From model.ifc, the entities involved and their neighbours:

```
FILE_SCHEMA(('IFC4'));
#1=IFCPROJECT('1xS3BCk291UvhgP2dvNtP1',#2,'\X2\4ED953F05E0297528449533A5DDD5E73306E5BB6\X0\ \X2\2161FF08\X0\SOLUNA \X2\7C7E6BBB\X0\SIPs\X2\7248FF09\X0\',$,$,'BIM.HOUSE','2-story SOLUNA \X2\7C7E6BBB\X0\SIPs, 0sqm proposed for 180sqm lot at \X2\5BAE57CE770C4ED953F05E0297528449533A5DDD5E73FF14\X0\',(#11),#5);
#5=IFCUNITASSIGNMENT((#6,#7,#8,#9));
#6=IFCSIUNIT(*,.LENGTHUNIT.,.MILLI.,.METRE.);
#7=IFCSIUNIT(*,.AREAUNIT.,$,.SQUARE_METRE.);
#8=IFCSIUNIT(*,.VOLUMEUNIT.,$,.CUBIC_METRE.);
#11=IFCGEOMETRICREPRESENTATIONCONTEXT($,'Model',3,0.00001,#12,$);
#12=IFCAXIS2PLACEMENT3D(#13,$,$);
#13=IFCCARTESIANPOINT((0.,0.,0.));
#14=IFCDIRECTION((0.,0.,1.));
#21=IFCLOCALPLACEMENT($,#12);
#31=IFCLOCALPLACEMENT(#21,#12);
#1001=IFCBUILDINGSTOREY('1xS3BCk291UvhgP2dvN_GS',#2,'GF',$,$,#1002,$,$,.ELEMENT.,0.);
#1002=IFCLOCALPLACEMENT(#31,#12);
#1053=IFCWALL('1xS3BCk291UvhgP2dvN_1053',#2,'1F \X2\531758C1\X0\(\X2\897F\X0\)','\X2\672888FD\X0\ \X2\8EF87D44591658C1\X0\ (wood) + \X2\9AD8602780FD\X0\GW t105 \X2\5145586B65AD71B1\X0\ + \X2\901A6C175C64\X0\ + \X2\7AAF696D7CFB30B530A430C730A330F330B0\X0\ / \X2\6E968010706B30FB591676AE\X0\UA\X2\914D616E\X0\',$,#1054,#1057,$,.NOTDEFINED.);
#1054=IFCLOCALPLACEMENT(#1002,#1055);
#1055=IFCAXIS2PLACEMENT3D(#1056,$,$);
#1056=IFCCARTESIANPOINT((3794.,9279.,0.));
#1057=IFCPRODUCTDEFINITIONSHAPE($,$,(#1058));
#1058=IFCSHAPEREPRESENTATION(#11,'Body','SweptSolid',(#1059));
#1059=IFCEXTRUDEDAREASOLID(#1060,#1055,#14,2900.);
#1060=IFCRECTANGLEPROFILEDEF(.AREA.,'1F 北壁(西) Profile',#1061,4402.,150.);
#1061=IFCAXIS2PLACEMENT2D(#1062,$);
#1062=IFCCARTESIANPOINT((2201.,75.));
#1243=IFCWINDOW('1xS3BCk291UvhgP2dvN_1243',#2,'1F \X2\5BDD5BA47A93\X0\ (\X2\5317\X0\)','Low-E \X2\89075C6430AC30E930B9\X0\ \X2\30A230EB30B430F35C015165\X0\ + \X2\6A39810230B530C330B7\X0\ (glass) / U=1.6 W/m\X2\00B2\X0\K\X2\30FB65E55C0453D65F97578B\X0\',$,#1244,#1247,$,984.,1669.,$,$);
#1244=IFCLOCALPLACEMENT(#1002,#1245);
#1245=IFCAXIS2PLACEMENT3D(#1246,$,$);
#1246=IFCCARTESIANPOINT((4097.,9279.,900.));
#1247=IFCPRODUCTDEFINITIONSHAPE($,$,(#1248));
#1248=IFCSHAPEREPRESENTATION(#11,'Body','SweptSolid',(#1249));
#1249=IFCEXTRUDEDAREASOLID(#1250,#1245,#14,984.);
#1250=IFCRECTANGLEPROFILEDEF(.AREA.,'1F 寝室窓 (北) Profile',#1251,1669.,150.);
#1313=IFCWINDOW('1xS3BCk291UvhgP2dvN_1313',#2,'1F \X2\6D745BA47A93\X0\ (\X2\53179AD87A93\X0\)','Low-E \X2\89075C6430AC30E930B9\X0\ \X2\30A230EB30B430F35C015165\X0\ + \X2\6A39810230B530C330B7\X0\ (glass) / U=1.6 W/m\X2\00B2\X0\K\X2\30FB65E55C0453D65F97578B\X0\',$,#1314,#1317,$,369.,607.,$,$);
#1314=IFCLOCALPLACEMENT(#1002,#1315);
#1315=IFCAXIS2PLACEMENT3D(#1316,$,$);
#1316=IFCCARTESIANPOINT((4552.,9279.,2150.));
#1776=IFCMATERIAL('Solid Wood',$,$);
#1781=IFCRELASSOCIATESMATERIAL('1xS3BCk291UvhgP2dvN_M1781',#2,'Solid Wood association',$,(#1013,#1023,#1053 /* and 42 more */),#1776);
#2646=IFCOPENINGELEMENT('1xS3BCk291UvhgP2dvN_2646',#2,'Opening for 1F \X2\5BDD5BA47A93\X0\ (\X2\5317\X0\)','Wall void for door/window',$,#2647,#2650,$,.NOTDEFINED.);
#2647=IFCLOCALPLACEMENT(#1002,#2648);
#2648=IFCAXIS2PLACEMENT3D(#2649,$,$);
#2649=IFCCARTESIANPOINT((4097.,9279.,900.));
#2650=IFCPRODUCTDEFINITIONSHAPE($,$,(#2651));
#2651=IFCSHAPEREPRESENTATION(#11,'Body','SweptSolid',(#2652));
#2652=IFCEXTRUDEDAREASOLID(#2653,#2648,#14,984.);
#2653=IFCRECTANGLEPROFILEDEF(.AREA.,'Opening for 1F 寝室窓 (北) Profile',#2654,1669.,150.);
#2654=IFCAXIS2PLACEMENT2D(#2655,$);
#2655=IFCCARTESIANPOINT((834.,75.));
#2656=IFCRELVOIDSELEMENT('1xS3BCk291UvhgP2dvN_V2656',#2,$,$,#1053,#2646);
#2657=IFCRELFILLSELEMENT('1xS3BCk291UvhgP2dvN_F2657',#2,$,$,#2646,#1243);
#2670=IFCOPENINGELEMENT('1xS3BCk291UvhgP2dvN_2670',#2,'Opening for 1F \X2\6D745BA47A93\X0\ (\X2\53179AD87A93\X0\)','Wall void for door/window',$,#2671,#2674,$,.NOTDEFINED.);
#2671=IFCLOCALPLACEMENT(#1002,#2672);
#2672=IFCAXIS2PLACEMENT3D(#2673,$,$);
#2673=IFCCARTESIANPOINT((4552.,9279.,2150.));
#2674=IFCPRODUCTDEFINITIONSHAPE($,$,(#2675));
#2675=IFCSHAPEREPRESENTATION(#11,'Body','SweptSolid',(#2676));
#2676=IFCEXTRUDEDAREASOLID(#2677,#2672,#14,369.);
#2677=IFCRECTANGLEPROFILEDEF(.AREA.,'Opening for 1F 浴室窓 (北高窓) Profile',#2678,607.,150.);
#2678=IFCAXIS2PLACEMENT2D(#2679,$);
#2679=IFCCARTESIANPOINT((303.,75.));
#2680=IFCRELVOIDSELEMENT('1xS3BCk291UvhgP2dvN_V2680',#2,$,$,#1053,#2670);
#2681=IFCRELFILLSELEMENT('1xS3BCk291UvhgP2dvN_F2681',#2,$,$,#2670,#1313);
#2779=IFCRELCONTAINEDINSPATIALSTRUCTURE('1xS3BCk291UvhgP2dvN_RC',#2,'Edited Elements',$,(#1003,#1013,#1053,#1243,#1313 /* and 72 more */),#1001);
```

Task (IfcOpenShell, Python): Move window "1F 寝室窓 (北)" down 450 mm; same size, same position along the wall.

```python
import numpy as np
import ifcopenshell
import ifcopenshell.api.geometry
import ifcopenshell.util.placement
import ifcopenshell.util.unit

model = ifcopenshell.open("model.ifc")
unit_scale = ifcopenshell.util.unit.calculate_unit_scale(model)

window = model.by_guid("1xS3BCk291UvhgP2dvN_1243")
opening = window.FillsVoids[0].RelatingOpeningElement
dz = -0.45 / unit_scale

shift = np.array([0.0, 0.0, dz])
# The window is not placed relative to its opening, so move both.
for product in (opening, window):
    matrix = ifcopenshell.util.placement.get_local_placement(product.ObjectPlacement)
    matrix[:3, 3] += shift
    ifcopenshell.api.geometry.edit_object_placement(model, product=product, matrix=matrix, is_si=False)

print(f"moved by {dz * unit_scale:+.3f} m")

model.write("model_rev.ifc")
```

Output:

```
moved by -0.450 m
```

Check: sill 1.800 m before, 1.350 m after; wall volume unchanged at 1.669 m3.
